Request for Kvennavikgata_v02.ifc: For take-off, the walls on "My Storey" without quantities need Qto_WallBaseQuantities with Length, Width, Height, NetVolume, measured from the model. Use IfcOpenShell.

First a look at what the model holds.

```python
import ifcopenshell
import ifcopenshell.util.element
import ifcopenshell.util.unit

model = ifcopenshell.open("Kvennavikgata_v02.ifc")
print(model.schema)
for unit_type in ("LENGTHUNIT", "AREAUNIT", "VOLUMEUNIT"):
    print(unit_type, ifcopenshell.util.unit.calculate_unit_scale(model, unit_type))
storey = next(s for s in model.by_type("IfcBuildingStorey") if s.Name == "My Storey")
walls = [e for e in ifcopenshell.util.element.get_decomposition(storey) if e.is_a("IfcWall")]
for e in sorted(walls, key=lambda e: e.id()):
    print(e.id(), e.is_a(), e.Name, list(ifcopenshell.util.element.get_psets(e, qtos_only=True)), sep=" | ")
```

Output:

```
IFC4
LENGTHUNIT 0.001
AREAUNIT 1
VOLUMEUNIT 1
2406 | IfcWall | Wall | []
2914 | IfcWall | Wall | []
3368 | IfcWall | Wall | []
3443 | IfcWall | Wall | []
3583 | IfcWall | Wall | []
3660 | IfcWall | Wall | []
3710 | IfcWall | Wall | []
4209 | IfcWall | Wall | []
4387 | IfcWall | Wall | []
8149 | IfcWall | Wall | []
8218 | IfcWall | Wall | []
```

```python
import ifcopenshell
import ifcopenshell.api.pset
import ifcopenshell.geom
import ifcopenshell.util.element
import ifcopenshell.util.shape
import ifcopenshell.util.unit

model = ifcopenshell.open("Kvennavikgata_v02.ifc")
unit_scale = ifcopenshell.util.unit.calculate_unit_scale(model)
volume_scale = ifcopenshell.util.unit.calculate_unit_scale(model, "VOLUMEUNIT")
settings = ifcopenshell.geom.settings()

storey = next(s for s in model.by_type("IfcBuildingStorey") if s.Name == "My Storey")
walls = [e for e in ifcopenshell.util.element.get_decomposition(storey) if e.is_a("IfcWall")]

for e in sorted(walls, key=lambda e: e.id()):
    if ifcopenshell.util.element.get_psets(e, qtos_only=True, should_inherit=False):
        continue
    # Geometry comes back in metres, in the element's own axes.
    shape = ifcopenshell.geom.create_shape(settings, e)
    values = {
        "Length": ifcopenshell.util.shape.get_x(shape.geometry) / unit_scale,
        "Width": ifcopenshell.util.shape.get_y(shape.geometry) / unit_scale,
        "Height": ifcopenshell.util.shape.get_z(shape.geometry) / unit_scale,
        "NetVolume": ifcopenshell.util.shape.get_volume(shape.geometry) / volume_scale,
    }
    qto = ifcopenshell.api.pset.add_qto(model, product=e, name="Qto_WallBaseQuantities")
    ifcopenshell.api.pset.edit_qto(model, qto=qto, properties=values)
    print(e.id(), {k: round(v, 3) for k, v in values.items()})

model.write("Kvennavikgata_v02_v2.ifc")
```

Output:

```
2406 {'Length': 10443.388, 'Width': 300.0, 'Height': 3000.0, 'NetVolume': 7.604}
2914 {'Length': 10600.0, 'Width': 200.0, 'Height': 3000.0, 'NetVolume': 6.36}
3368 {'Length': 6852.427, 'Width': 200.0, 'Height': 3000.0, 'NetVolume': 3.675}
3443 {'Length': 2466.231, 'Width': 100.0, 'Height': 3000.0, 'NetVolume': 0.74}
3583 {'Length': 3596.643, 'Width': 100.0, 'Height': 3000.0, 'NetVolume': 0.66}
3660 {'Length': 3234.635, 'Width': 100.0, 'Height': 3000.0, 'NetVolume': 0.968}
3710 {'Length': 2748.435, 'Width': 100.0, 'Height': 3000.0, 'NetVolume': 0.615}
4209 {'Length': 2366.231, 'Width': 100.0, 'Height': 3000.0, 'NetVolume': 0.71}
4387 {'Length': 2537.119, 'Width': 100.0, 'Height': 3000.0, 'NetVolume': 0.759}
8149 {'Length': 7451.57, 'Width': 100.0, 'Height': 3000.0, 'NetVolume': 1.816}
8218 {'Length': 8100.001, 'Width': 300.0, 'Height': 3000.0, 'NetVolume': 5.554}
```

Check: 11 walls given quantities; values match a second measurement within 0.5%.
